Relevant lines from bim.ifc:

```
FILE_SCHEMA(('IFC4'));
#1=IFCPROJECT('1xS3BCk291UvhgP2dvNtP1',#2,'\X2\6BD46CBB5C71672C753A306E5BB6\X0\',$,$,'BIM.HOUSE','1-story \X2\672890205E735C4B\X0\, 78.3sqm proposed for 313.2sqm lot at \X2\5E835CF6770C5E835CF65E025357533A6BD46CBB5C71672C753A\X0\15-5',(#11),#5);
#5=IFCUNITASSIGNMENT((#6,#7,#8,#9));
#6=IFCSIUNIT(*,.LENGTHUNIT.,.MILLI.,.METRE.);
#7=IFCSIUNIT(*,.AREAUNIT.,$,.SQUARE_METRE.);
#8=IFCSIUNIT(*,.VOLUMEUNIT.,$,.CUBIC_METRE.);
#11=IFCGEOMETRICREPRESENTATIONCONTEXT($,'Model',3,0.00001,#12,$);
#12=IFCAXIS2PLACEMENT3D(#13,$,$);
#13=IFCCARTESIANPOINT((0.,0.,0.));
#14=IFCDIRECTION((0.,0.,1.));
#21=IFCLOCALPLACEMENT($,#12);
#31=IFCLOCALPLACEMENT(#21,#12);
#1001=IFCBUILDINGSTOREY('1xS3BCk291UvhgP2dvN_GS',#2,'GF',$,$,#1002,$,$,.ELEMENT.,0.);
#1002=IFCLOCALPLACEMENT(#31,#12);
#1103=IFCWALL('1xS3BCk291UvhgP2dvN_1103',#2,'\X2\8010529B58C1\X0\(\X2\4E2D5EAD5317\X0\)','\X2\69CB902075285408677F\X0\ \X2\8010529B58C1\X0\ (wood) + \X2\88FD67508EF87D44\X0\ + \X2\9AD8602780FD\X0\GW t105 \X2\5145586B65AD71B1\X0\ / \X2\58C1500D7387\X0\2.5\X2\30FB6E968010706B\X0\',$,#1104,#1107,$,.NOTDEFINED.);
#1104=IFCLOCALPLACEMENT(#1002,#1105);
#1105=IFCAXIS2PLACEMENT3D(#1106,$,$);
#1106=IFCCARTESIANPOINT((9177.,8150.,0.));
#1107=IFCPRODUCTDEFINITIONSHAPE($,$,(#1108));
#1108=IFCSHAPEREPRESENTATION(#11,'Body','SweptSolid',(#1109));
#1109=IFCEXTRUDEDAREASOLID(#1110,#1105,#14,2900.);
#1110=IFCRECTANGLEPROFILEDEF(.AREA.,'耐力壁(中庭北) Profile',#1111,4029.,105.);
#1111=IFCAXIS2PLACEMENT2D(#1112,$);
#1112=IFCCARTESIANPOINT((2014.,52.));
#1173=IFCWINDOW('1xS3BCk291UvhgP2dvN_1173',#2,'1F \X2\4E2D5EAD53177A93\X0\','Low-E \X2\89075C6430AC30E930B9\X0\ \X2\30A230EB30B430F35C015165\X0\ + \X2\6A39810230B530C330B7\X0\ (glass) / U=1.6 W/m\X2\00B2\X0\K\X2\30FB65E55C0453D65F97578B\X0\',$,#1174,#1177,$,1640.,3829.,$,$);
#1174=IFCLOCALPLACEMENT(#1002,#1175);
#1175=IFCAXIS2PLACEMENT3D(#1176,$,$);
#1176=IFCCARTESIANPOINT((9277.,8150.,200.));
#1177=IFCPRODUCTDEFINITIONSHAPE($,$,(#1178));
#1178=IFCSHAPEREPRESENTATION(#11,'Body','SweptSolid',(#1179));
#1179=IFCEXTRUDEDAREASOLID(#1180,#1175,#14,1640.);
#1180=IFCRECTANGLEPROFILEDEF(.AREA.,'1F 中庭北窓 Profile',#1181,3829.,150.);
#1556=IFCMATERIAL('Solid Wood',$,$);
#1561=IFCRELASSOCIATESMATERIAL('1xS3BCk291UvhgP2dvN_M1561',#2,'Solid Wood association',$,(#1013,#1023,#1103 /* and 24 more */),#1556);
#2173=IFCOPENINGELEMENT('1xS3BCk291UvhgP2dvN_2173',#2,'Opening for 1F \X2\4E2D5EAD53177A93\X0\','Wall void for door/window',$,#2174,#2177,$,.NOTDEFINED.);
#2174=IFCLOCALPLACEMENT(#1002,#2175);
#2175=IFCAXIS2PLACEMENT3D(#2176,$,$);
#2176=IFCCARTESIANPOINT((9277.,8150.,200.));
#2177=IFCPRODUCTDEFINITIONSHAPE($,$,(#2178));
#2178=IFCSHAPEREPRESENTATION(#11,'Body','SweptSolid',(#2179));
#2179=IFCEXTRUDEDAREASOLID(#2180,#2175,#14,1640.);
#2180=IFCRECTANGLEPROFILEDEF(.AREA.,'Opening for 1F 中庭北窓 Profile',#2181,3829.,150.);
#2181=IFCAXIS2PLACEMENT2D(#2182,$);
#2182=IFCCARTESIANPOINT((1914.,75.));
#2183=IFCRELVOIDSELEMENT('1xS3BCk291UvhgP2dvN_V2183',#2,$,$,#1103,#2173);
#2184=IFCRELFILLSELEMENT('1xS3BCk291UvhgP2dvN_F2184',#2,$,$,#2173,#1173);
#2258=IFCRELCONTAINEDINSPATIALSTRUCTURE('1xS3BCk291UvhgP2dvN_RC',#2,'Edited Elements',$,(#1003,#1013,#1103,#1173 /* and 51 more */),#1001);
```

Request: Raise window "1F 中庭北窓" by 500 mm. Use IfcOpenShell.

```python
import numpy as np
import ifcopenshell
import ifcopenshell.api.geometry
import ifcopenshell.util.placement
import ifcopenshell.util.unit

model = ifcopenshell.open("bim.ifc")
unit_scale = ifcopenshell.util.unit.calculate_unit_scale(model)

window = model.by_guid("1xS3BCk291UvhgP2dvN_1173")
opening = window.FillsVoids[0].RelatingOpeningElement
dz = 0.5 / unit_scale

shift = np.array([0.0, 0.0, dz])
# The window is not placed relative to its opening, so move both.
for product in (opening, window):
    matrix = ifcopenshell.util.placement.get_local_placement(product.ObjectPlacement)
    matrix[:3, 3] += shift
    ifcopenshell.api.geometry.edit_object_placement(model, product=product, matrix=matrix, is_si=False)

print(f"moved by {dz * unit_scale:+.3f} m")

model.write("bim_edited.ifc")
```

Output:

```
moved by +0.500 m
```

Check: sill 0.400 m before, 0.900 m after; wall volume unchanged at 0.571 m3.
